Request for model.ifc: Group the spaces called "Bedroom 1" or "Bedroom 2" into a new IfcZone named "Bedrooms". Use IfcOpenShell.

First a look at what the model holds.

```python
import ifcopenshell

model = ifcopenshell.open("model.ifc")
print(model.schema)
seen = {}
for space in model.by_type("IfcSpace"):
    seen[space.LongName] = seen.get(space.LongName, 0) + 1
for name, count in sorted(seen.items(), key=str):
    print(count, "x", name)
print("zones:", [z.Name for z in model.by_type("IfcZone")][:20])
```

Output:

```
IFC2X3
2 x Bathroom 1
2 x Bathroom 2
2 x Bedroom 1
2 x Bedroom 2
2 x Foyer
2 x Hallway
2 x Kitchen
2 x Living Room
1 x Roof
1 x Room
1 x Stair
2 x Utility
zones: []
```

```python
import ifcopenshell
import ifcopenshell.api.group
import ifcopenshell.api.root

model = ifcopenshell.open("model.ifc")

names = {"Bedroom 1", "Bedroom 2"}
spaces = [s for s in model.by_type("IfcSpace") if s.LongName in names]

zone = ifcopenshell.api.root.create_entity(model, ifc_class="IfcZone", name="Bedrooms")
ifcopenshell.api.group.assign_group(model, products=spaces, group=zone)
print(len(spaces), "spaces in", zone.Name)

model.write("model_rev.ifc")
```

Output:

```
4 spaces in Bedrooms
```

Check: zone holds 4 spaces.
